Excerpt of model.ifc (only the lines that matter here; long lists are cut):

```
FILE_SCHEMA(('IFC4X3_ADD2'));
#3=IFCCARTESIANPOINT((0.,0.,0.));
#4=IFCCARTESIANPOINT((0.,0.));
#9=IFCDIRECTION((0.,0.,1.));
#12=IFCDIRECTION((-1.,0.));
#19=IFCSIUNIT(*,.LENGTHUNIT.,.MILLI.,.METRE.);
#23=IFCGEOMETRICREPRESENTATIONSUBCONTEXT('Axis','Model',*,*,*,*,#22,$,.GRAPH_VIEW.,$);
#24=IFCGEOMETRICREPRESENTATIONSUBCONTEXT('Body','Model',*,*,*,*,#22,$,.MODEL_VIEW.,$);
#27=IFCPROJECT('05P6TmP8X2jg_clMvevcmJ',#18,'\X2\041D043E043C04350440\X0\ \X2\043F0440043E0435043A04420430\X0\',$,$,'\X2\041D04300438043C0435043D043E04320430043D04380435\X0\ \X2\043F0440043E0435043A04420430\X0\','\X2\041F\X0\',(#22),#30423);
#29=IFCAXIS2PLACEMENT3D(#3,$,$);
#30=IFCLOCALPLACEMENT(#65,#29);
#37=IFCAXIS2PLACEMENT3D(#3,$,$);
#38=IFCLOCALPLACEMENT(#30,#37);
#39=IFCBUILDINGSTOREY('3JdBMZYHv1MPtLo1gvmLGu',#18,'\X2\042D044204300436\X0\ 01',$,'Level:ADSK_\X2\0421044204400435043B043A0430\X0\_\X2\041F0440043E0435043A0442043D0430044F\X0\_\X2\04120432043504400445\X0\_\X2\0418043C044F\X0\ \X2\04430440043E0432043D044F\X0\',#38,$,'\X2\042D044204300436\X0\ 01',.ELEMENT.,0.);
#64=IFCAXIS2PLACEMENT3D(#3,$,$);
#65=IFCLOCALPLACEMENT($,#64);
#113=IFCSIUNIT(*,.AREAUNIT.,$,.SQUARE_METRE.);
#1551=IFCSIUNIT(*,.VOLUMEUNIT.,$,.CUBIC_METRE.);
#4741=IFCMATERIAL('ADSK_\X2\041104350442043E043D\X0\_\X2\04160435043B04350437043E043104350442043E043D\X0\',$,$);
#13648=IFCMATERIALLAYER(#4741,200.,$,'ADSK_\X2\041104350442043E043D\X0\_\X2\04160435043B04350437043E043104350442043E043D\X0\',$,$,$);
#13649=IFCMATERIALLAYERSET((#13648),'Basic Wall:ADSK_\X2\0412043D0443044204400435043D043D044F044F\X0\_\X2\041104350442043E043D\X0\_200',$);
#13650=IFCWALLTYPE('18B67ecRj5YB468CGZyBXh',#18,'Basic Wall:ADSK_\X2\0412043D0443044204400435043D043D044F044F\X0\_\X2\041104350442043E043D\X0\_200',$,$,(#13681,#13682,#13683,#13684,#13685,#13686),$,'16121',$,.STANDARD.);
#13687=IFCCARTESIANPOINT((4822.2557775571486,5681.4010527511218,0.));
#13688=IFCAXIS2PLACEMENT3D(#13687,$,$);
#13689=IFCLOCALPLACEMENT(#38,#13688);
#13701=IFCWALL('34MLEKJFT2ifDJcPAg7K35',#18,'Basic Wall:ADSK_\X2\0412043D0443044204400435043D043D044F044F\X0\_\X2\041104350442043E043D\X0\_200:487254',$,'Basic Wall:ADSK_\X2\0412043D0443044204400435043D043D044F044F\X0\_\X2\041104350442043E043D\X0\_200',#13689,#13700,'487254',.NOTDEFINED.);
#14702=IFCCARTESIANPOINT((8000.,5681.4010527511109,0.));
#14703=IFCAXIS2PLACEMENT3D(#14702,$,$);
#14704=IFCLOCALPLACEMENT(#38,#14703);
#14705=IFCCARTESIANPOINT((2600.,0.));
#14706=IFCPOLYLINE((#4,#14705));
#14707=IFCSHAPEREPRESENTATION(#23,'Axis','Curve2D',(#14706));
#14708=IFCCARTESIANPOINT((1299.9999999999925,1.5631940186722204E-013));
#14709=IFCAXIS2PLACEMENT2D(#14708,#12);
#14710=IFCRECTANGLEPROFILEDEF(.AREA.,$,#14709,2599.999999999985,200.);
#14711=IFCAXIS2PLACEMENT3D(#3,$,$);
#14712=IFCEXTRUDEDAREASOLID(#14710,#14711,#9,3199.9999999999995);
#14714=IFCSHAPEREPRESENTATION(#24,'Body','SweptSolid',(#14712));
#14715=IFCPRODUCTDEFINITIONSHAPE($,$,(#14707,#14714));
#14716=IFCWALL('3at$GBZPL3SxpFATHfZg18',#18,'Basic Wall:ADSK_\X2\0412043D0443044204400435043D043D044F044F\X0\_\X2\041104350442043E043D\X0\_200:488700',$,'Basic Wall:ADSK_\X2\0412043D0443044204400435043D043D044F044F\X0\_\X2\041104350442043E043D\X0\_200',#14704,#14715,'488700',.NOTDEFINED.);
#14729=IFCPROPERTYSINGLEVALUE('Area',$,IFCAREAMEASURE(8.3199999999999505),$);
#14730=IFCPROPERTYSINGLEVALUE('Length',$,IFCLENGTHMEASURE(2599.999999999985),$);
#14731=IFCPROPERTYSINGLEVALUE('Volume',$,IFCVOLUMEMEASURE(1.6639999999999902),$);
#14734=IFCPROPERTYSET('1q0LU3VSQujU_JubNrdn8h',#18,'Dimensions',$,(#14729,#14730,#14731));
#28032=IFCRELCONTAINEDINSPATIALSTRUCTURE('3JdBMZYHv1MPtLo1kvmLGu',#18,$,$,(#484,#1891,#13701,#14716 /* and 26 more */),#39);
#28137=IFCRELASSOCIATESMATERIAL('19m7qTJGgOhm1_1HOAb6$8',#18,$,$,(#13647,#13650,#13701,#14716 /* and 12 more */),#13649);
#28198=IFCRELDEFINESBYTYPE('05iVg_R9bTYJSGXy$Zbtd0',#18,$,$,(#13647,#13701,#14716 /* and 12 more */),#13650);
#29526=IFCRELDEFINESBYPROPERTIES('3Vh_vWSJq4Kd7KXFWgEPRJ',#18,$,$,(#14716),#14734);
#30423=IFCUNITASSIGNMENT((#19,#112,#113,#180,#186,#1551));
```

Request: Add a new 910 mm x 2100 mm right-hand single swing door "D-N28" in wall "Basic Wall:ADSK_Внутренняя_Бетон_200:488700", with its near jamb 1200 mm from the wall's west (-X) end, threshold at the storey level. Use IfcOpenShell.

```python
import numpy as np
import ifcopenshell
import ifcopenshell.api.feature
import ifcopenshell.api.geometry
import ifcopenshell.api.pset
import ifcopenshell.api.root
import ifcopenshell.api.spatial
import ifcopenshell.geom
import ifcopenshell.util.element
import ifcopenshell.util.placement
import ifcopenshell.util.representation
import ifcopenshell.util.shape
import ifcopenshell.util.unit

model = ifcopenshell.open("model.ifc")
unit_scale = ifcopenshell.util.unit.calculate_unit_scale(model)
area_scale = ifcopenshell.util.unit.calculate_unit_scale(model, "AREAUNIT")
volume_scale = ifcopenshell.util.unit.calculate_unit_scale(model, "VOLUMEUNIT")
settings = ifcopenshell.geom.settings()


def volume(element):
    """Net volume in cubic metres, openings subtracted."""
    shape = ifcopenshell.geom.create_shape(settings, element)
    return ifcopenshell.util.shape.get_volume(shape.geometry)


wall = model.by_guid("3at$GBZPL3SxpFATHfZg18")
storey = ifcopenshell.util.element.get_container(wall, ifc_class="IfcBuildingStorey")
context = ifcopenshell.util.representation.get_context(model, "Model", "Body", "MODEL_VIEW")
before = volume(wall)

width, height, from_end, sill = 0.91, 2.1, 1.2, 0.0  # metres

# The wall runs along its own X axis, and the end named is its -X end.
wall_shape = ifcopenshell.geom.create_shape(settings, wall)
x, y, z = ifcopenshell.util.shape.get_vertices(wall_shape.geometry).T
start = x.min() + from_end
face, thickness = float(y.min()), float(y.max() - y.min())
wall_matrix = ifcopenshell.util.placement.get_local_placement(wall.ObjectPlacement)
level = ifcopenshell.util.placement.get_local_placement(storey.ObjectPlacement)[2, 3]


def in_wall(x, y):
    """Placement at x, y metres in the wall's axes, at sill height."""
    matrix = wall_matrix.copy()
    matrix[:, 3] = wall_matrix @ np.array([x / unit_scale, y / unit_scale, 0.0, 1.0])
    matrix[2, 3] = level + sill / unit_scale
    return matrix


# Opening: a box that overshoots both wall faces by 50 mm.
opening = ifcopenshell.api.root.create_entity(model, ifc_class="IfcOpeningElement", predefined_type="OPENING")
box = ifcopenshell.api.geometry.add_wall_representation(
    model, context=context, length=width, height=height, thickness=thickness + 0.1
)
ifcopenshell.api.geometry.assign_representation(model, product=opening, representation=box)
ifcopenshell.api.geometry.edit_object_placement(model, product=opening, matrix=in_wall(start, face - 0.05), is_si=False)
ifcopenshell.api.feature.add_feature(model, feature=opening, element=wall)

door = ifcopenshell.api.root.create_entity(model, ifc_class="IfcDoor", name="D-N28", predefined_type="DOOR")
door.OverallWidth, door.OverallHeight = width / unit_scale, height / unit_scale
door.OperationType = "SINGLE_SWING_RIGHT"
body = ifcopenshell.api.geometry.add_door_representation(
    model,
    context=context,
    overall_width=door.OverallWidth,
    overall_height=door.OverallHeight,
    operation_type="SINGLE_SWING_RIGHT",
    lining_properties={"LiningDepth": thickness / unit_scale, "ThresholdDepth": thickness / unit_scale},
)
ifcopenshell.api.geometry.assign_representation(model, product=door, representation=body)
ifcopenshell.api.spatial.assign_container(model, products=[door], relating_structure=storey)
ifcopenshell.api.feature.add_filling(model, opening=opening, element=door)

# The lining spans the wall, so the door starts at the wall face.
ifcopenshell.api.geometry.edit_object_placement(model, product=door, matrix=in_wall(start, face), is_si=False)

after = volume(wall)

# Update the wall's stored quantities.
pset = model.by_id(ifcopenshell.util.element.get_pset(wall, "Dimensions", should_inherit=False)["id"])
ifcopenshell.api.pset.edit_pset(model, pset=pset, properties={
    "Area": model.create_entity("IfcAreaMeasure", after / thickness / area_scale),
    "Volume": model.create_entity("IfcVolumeMeasure", after / volume_scale),
})

print(f"wall volume {before:.3f} -> {after:.3f} m3")

model.write("model_rev.ifc")
```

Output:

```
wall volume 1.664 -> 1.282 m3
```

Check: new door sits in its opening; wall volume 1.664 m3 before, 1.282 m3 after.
